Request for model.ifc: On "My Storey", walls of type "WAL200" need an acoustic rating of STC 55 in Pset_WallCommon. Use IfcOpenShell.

First a look at what the model holds.

```python
import ifcopenshell
import ifcopenshell.util.element

model = ifcopenshell.open("model.ifc")
print(model.schema)
storey = next(s for s in model.by_type("IfcBuildingStorey") if s.Name == "My Storey")
walls = [e for e in ifcopenshell.util.element.get_decomposition(storey) if e.is_a("IfcWall")]
seen = {}
for e in walls:
    element_type = ifcopenshell.util.element.get_type(e)
    key = (element_type.Name if element_type != e and element_type else None, ifcopenshell.util.element.get_pset(e, "Pset_WallCommon", "AcousticRating"))
    seen[key] = seen.get(key, 0) + 1
for (name, value), count in sorted(seen.items(), key=str):
    print(count, "x", name, "|", value)
```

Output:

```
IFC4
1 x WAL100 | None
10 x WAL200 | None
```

```python
import ifcopenshell
import ifcopenshell.api.pset
import ifcopenshell.util.element

model = ifcopenshell.open("model.ifc")

storey = next(s for s in model.by_type("IfcBuildingStorey") if s.Name == "My Storey")
walls = [e for e in ifcopenshell.util.element.get_decomposition(storey) if e.is_a("IfcWall")]

count = 0
for e in walls:
    element_type = ifcopenshell.util.element.get_type(e)
    if element_type in (None, e) or element_type.Name != "WAL200":
        continue
    # add_pset returns the element's existing set when there is one.
    pset = ifcopenshell.api.pset.add_pset(model, product=e, name="Pset_WallCommon")
    ifcopenshell.api.pset.edit_pset(model, pset=pset, properties={"AcousticRating": "STC 55"})
    count += 1

print(count, "walls updated")

model.write("model-out.ifc")
```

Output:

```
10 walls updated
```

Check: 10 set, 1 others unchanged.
